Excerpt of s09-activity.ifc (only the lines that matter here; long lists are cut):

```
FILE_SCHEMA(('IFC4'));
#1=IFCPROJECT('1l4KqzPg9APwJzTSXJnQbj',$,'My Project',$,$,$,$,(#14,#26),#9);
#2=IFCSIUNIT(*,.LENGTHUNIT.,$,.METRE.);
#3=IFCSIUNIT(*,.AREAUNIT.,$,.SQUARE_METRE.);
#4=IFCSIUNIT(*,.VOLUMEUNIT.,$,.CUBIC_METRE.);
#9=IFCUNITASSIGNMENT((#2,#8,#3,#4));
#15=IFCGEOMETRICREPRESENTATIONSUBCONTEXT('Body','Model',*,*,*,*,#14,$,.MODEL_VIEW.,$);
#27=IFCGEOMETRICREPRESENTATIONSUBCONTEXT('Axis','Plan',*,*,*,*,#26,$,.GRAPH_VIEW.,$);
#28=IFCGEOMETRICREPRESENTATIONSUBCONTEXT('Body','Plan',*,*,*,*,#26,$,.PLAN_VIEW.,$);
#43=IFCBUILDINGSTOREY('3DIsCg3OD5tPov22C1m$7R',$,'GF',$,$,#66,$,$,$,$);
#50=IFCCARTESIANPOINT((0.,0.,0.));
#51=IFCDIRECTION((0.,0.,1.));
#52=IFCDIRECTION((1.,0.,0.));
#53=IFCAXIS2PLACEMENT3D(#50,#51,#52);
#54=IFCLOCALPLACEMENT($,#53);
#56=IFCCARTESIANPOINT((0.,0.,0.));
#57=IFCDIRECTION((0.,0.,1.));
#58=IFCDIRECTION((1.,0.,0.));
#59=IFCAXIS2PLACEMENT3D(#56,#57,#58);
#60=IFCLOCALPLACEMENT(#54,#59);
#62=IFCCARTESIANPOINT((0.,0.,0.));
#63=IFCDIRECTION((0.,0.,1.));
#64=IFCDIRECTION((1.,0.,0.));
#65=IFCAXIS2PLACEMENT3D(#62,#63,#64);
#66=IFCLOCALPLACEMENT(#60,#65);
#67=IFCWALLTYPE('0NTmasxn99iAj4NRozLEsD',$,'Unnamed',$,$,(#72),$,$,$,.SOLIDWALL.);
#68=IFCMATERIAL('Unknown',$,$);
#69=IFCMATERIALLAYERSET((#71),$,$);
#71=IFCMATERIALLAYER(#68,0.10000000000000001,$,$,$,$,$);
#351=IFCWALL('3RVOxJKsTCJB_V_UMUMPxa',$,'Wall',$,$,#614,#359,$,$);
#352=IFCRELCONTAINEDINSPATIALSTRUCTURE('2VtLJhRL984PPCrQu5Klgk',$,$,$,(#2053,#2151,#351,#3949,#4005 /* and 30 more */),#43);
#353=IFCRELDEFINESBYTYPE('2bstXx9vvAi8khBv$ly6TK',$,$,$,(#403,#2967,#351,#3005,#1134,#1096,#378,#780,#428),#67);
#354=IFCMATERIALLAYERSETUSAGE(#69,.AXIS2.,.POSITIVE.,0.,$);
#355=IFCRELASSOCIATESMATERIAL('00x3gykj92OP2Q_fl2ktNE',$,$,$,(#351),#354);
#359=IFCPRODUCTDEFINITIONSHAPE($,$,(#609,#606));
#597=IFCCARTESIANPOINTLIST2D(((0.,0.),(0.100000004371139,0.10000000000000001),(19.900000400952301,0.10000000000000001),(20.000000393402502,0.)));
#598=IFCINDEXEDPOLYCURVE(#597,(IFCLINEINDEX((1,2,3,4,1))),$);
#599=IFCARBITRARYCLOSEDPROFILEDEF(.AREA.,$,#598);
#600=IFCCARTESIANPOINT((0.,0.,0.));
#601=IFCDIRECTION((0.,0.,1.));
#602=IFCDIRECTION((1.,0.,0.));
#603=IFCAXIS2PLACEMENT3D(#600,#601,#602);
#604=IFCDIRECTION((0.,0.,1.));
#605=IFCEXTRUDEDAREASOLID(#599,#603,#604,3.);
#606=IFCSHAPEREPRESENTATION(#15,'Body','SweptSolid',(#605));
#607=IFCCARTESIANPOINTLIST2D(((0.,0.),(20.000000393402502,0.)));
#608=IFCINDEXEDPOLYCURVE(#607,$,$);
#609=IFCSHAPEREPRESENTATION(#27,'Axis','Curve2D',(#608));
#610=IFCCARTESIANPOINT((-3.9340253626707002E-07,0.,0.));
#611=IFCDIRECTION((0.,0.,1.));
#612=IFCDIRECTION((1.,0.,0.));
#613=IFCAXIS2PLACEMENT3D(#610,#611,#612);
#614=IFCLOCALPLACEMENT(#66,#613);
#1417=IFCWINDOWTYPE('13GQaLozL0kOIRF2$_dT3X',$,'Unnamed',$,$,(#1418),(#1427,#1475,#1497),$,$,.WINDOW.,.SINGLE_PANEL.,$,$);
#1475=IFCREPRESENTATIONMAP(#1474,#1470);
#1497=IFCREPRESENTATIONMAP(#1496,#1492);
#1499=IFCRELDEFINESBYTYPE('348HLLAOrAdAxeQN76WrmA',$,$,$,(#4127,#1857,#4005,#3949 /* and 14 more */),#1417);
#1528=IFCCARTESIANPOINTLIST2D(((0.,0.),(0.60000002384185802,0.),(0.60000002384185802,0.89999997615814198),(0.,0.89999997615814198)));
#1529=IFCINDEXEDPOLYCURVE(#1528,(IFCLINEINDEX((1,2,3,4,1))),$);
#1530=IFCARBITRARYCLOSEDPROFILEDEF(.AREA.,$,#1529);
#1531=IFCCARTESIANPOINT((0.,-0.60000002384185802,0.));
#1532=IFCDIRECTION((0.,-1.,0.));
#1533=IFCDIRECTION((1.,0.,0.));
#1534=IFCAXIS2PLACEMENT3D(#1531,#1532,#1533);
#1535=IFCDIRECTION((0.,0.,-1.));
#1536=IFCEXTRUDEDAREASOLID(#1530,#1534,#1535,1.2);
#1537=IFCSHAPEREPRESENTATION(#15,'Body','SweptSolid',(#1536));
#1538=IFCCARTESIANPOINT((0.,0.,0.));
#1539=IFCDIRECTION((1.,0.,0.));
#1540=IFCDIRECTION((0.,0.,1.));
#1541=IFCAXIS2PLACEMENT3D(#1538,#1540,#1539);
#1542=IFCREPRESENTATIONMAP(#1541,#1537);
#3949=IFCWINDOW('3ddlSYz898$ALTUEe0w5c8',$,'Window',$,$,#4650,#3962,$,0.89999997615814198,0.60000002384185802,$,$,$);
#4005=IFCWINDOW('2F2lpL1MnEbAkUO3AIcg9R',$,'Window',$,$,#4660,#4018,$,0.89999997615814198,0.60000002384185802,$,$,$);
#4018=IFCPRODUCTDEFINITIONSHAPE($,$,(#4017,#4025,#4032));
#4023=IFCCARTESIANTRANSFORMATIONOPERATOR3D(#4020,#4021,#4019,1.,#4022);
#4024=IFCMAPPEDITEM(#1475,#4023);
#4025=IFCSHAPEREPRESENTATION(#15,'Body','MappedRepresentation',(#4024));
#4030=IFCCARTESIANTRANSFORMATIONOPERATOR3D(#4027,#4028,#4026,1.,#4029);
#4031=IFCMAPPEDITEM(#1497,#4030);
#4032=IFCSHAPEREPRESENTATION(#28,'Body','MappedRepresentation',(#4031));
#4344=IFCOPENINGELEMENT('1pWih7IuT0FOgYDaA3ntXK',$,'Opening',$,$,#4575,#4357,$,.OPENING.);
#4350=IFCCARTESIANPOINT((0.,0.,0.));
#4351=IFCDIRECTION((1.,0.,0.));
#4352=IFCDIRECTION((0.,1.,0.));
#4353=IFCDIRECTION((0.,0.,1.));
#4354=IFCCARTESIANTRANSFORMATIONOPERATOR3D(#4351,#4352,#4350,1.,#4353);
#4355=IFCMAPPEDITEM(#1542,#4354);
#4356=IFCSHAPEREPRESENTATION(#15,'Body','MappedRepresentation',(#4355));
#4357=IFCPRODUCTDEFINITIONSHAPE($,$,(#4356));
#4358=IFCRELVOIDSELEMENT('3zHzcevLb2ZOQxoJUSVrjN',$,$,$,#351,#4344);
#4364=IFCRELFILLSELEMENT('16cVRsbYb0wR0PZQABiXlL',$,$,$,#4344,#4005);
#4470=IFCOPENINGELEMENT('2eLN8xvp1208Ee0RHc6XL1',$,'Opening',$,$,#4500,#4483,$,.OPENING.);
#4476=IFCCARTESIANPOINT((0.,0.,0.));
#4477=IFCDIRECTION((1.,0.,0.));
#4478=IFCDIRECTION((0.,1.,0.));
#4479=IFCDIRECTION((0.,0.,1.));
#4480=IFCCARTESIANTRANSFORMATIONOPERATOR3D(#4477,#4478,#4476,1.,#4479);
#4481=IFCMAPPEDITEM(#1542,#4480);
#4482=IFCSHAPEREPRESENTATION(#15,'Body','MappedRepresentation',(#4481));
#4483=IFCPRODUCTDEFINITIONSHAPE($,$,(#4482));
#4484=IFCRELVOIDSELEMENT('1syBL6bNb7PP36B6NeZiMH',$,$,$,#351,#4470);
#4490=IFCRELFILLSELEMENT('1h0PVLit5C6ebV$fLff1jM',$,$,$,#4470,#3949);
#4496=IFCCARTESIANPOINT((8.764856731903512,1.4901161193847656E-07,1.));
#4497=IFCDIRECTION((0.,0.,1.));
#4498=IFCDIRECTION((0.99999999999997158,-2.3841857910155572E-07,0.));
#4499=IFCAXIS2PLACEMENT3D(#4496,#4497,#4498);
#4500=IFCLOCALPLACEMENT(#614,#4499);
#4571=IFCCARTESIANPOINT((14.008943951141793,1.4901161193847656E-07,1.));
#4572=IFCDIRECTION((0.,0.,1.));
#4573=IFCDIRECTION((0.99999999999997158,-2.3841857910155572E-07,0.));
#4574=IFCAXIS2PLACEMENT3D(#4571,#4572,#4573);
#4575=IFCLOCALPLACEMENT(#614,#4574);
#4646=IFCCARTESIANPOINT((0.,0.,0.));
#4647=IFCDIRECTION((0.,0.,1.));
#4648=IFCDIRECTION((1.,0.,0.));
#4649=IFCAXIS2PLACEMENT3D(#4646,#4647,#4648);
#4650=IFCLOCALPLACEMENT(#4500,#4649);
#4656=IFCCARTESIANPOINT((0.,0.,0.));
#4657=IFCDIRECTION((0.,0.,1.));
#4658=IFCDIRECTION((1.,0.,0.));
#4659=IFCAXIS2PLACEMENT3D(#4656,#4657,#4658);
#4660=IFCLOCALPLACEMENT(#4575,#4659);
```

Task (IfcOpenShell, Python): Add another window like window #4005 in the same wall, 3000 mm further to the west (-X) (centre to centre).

```python
import ifcopenshell
import ifcopenshell.api.feature
import ifcopenshell.api.geometry
import ifcopenshell.api.root
import ifcopenshell.geom
import ifcopenshell.util.element
import ifcopenshell.util.placement
import ifcopenshell.util.shape

model = ifcopenshell.open("s09-activity.ifc")
settings = ifcopenshell.geom.settings()


def volume(element):
    """Net volume in cubic metres, openings subtracted."""
    shape = ifcopenshell.geom.create_shape(settings, element)
    return ifcopenshell.util.shape.get_volume(shape.geometry)


window = model.by_guid("2F2lpL1MnEbAkUO3AIcg9R")
opening = window.FillsVoids[0].RelatingOpeningElement
wall = opening.VoidsElements[0].RelatingBuildingElement
before = volume(wall)
shift = ifcopenshell.util.placement.get_local_placement(wall.ObjectPlacement)[:3, 0] * -3.0

# copy_class copies the void relationship, type, container and properties, but no geometry.
new_opening = ifcopenshell.api.root.copy_class(model, product=opening)
new_opening.Representation = ifcopenshell.util.element.copy_deep(
    model, opening.Representation, exclude=["IfcGeometricRepresentationContext", "IfcRepresentationMap"]
)
new_window = ifcopenshell.api.root.copy_class(model, product=window)
new_window.Representation = ifcopenshell.util.element.copy_deep(
    model, window.Representation, exclude=["IfcGeometricRepresentationContext", "IfcRepresentationMap"]
)
ifcopenshell.api.feature.add_filling(model, opening=new_opening, element=new_window)

for old, new in ((opening, new_opening), (window, new_window)):
    matrix = ifcopenshell.util.placement.get_local_placement(old.ObjectPlacement)
    matrix[:3, 3] += shift
    ifcopenshell.api.geometry.edit_object_placement(model, product=new, matrix=matrix, is_si=False)

after = volume(wall)

print(f"wall volume {before:.3f} -> {after:.3f} m3")

model.write("s09-activity_edited.ifc")
```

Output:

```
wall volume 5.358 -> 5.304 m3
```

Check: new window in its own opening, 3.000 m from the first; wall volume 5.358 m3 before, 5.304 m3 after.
